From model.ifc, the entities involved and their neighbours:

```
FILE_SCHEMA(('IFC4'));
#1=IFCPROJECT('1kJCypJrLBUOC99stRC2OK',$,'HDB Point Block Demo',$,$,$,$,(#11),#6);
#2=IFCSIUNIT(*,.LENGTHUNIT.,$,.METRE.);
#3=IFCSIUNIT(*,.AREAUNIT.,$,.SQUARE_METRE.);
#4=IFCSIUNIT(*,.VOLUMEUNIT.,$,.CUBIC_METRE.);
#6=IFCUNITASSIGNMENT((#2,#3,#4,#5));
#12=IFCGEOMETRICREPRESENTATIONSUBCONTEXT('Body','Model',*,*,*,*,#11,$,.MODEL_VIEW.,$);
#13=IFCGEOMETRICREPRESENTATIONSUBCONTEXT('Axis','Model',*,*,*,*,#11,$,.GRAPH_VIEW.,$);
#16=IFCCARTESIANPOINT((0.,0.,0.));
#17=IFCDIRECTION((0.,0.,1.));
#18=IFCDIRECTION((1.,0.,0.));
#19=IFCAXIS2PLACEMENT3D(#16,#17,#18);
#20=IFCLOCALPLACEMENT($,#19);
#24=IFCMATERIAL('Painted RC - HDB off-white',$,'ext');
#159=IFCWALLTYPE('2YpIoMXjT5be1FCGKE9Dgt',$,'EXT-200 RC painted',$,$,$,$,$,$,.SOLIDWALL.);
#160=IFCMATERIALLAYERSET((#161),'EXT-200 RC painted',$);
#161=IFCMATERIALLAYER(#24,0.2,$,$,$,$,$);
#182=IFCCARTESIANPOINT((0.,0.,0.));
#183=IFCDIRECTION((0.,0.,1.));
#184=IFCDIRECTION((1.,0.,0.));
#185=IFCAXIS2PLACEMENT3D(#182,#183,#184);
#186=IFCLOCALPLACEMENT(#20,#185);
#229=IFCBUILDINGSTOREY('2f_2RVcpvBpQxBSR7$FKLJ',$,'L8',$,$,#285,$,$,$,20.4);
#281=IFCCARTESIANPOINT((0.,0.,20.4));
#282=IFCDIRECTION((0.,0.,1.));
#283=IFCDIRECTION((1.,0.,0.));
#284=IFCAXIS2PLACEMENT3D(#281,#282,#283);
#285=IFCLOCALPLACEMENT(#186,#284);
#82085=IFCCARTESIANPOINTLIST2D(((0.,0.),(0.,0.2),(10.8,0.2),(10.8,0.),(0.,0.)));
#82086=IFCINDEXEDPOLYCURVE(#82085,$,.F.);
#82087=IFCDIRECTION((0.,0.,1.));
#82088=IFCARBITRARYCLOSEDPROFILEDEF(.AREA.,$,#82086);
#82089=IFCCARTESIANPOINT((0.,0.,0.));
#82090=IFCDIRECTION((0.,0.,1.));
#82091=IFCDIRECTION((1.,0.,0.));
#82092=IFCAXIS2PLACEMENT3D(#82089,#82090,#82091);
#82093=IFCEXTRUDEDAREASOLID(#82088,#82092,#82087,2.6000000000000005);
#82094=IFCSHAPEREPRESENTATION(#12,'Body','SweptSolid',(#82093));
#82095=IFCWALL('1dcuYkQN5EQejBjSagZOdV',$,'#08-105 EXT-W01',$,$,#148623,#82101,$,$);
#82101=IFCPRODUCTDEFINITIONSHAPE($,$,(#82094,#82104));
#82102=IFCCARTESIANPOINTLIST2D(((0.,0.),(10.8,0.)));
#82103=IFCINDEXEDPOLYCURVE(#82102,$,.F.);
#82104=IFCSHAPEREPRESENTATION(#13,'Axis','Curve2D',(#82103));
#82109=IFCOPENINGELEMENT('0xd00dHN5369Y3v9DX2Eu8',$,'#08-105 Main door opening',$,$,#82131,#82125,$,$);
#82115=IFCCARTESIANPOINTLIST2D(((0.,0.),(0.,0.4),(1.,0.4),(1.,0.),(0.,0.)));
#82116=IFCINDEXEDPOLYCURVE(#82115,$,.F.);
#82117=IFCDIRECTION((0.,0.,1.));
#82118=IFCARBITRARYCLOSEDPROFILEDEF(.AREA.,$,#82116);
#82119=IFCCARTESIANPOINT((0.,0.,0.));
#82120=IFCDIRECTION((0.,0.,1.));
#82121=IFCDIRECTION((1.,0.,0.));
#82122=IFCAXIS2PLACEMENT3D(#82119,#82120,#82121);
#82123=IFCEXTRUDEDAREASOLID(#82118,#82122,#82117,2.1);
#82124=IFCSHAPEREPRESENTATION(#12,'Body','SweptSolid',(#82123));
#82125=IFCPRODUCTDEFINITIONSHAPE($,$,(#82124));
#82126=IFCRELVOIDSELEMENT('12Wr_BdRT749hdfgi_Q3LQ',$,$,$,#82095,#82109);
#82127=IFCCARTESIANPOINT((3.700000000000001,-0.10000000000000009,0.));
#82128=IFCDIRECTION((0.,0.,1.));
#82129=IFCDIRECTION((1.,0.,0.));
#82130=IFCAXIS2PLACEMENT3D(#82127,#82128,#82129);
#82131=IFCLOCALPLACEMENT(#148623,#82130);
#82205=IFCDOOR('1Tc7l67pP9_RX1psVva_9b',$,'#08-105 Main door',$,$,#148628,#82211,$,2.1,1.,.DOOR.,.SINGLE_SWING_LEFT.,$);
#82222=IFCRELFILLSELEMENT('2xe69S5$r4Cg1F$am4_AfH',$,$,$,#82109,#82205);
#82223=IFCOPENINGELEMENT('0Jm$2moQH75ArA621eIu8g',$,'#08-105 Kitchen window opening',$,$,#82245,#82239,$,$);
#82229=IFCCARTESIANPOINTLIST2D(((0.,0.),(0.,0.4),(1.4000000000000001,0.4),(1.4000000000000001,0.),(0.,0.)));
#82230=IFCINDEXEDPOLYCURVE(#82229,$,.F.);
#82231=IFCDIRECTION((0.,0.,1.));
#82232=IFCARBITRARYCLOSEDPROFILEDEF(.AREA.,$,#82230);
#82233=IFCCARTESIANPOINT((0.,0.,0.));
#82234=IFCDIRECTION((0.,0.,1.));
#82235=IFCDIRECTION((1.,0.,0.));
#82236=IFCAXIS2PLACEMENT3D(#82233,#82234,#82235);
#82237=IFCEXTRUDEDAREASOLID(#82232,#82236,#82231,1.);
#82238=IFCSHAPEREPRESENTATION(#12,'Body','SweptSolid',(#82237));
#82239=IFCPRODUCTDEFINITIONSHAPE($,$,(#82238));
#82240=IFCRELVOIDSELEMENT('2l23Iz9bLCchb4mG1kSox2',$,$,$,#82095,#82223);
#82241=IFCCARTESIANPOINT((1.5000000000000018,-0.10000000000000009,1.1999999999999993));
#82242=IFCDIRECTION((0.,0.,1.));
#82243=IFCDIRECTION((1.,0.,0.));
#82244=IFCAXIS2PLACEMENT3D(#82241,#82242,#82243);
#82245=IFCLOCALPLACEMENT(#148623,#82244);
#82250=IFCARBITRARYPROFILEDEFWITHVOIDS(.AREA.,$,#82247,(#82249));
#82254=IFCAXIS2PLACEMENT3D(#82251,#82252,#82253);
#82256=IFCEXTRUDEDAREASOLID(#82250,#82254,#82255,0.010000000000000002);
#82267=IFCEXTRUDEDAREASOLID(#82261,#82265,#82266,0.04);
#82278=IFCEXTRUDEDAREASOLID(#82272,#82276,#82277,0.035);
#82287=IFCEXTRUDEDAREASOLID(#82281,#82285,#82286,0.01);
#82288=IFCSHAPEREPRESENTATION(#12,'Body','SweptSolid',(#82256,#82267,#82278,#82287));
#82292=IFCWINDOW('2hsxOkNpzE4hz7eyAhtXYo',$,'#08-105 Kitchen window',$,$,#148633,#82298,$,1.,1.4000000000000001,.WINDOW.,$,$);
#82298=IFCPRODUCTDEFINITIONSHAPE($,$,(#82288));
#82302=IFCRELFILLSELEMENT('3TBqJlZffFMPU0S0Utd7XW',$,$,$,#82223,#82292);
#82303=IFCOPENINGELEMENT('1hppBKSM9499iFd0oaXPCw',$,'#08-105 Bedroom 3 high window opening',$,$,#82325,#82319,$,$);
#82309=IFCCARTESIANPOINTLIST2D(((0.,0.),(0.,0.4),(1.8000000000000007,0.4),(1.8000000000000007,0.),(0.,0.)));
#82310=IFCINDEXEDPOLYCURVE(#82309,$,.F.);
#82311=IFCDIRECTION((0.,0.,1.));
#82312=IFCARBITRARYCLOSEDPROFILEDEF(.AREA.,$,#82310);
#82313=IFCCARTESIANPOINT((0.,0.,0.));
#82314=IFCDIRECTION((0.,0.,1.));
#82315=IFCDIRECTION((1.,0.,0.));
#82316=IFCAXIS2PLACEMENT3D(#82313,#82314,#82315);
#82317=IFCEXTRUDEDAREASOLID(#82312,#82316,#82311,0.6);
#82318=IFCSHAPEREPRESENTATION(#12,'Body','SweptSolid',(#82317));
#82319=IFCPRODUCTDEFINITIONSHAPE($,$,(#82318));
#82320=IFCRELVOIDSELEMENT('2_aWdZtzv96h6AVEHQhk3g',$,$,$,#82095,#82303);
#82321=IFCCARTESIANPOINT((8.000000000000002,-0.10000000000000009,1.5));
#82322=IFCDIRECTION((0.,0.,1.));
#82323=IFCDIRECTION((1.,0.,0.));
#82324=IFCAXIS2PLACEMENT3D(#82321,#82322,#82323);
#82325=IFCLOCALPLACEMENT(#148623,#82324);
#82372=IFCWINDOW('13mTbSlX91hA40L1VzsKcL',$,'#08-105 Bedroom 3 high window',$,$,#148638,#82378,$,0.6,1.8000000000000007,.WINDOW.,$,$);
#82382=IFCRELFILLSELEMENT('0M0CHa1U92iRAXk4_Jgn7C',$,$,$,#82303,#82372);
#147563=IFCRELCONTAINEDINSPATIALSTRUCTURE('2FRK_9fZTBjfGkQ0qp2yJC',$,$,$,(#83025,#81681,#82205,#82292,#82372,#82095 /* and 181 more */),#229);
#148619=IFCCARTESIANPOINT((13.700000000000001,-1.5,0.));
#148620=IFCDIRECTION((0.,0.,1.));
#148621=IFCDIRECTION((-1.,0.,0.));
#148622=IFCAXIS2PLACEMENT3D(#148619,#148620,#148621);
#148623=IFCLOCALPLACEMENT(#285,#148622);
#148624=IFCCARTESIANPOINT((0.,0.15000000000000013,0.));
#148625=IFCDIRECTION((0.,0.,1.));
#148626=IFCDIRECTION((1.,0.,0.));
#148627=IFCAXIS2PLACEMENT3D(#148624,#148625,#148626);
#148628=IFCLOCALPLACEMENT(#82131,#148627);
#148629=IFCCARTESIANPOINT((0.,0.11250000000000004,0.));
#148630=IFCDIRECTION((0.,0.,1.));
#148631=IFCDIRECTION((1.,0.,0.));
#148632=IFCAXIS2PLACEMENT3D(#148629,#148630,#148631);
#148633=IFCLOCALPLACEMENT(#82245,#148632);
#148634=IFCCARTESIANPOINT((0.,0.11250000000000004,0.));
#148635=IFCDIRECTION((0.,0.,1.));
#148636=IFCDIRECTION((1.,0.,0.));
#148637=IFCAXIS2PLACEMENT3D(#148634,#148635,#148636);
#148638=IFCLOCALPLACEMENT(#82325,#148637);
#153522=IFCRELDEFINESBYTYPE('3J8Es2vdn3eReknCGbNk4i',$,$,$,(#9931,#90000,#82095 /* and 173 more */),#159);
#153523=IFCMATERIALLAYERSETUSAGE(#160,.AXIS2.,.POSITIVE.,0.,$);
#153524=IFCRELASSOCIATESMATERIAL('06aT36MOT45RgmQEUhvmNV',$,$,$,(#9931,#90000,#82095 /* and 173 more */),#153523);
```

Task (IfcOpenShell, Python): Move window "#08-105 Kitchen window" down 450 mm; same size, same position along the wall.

```python
import numpy as np
import ifcopenshell
import ifcopenshell.api.geometry
import ifcopenshell.util.placement
import ifcopenshell.util.unit

model = ifcopenshell.open("model.ifc")
unit_scale = ifcopenshell.util.unit.calculate_unit_scale(model)

window = model.by_id(82292)
opening = window.FillsVoids[0].RelatingOpeningElement
dz = -0.45

shift = np.array([0.0, 0.0, dz])
# The window is placed relative to its opening, so it follows when the opening moves.
matrix = ifcopenshell.util.placement.get_local_placement(opening.ObjectPlacement)
matrix[:3, 3] += shift
ifcopenshell.api.geometry.edit_object_placement(
    model, product=opening, matrix=matrix, is_si=False, should_transform_children=True
)

print(f"moved by {dz * unit_scale:+.3f} m")

model.write("model_rev.ifc")
```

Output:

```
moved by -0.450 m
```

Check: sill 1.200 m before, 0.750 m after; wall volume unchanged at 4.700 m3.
